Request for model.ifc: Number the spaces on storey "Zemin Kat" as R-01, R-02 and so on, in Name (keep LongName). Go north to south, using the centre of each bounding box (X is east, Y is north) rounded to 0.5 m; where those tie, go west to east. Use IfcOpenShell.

First a look at what the model holds.

```python
import ifcopenshell
import ifcopenshell.util.element
import ifcopenshell.util.placement

model = ifcopenshell.open("model.ifc")
print(model.schema)
storey = next(s for s in model.by_type("IfcBuildingStorey") if s.Name == "Zemin Kat")
spaces = [e for e in ifcopenshell.util.element.get_decomposition(storey) if e.is_a("IfcSpace")]
for e in sorted(spaces, key=lambda e: e.id()):
    origin = ifcopenshell.util.placement.get_local_placement(e.ObjectPlacement)[:3, 3]
    print(e.id(), e.Name, e.LongName, origin.round(2) + 0.0, sep=" | ")
```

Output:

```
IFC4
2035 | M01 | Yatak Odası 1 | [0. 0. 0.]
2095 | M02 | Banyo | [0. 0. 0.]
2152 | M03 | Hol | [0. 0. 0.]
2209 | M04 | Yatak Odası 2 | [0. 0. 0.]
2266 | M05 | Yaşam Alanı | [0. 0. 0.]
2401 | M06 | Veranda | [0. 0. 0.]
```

```python
import ifcopenshell
import ifcopenshell.geom
import ifcopenshell.util.element
import ifcopenshell.util.shape

model = ifcopenshell.open("model.ifc")
settings = ifcopenshell.geom.settings()
settings.set("use-world-coords", True)


def centre(element):
    shape = ifcopenshell.geom.create_shape(settings, element)
    return ifcopenshell.util.shape.get_bbox_centroid(shape.geometry)


storey = next(s for s in model.by_type("IfcBuildingStorey") if s.Name == "Zemin Kat")
spaces = [e for e in ifcopenshell.util.element.get_decomposition(storey) if e.is_a("IfcSpace")]

# Insertion points can sit at a corner or the storey origin, so sort by the geometry (in metres).
centres = {e: centre(e) for e in spaces}
spaces.sort(key=lambda e: (-round(centres[e][1] / 0.5), centres[e][0]))

for i, e in enumerate(spaces, start=1):
    number = f"R-{i:02d}"
    e.Name = number
    print(e.id(), number)

model.write("model-out.ifc")
```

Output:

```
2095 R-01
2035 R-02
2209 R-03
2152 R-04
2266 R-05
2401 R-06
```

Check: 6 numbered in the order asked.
